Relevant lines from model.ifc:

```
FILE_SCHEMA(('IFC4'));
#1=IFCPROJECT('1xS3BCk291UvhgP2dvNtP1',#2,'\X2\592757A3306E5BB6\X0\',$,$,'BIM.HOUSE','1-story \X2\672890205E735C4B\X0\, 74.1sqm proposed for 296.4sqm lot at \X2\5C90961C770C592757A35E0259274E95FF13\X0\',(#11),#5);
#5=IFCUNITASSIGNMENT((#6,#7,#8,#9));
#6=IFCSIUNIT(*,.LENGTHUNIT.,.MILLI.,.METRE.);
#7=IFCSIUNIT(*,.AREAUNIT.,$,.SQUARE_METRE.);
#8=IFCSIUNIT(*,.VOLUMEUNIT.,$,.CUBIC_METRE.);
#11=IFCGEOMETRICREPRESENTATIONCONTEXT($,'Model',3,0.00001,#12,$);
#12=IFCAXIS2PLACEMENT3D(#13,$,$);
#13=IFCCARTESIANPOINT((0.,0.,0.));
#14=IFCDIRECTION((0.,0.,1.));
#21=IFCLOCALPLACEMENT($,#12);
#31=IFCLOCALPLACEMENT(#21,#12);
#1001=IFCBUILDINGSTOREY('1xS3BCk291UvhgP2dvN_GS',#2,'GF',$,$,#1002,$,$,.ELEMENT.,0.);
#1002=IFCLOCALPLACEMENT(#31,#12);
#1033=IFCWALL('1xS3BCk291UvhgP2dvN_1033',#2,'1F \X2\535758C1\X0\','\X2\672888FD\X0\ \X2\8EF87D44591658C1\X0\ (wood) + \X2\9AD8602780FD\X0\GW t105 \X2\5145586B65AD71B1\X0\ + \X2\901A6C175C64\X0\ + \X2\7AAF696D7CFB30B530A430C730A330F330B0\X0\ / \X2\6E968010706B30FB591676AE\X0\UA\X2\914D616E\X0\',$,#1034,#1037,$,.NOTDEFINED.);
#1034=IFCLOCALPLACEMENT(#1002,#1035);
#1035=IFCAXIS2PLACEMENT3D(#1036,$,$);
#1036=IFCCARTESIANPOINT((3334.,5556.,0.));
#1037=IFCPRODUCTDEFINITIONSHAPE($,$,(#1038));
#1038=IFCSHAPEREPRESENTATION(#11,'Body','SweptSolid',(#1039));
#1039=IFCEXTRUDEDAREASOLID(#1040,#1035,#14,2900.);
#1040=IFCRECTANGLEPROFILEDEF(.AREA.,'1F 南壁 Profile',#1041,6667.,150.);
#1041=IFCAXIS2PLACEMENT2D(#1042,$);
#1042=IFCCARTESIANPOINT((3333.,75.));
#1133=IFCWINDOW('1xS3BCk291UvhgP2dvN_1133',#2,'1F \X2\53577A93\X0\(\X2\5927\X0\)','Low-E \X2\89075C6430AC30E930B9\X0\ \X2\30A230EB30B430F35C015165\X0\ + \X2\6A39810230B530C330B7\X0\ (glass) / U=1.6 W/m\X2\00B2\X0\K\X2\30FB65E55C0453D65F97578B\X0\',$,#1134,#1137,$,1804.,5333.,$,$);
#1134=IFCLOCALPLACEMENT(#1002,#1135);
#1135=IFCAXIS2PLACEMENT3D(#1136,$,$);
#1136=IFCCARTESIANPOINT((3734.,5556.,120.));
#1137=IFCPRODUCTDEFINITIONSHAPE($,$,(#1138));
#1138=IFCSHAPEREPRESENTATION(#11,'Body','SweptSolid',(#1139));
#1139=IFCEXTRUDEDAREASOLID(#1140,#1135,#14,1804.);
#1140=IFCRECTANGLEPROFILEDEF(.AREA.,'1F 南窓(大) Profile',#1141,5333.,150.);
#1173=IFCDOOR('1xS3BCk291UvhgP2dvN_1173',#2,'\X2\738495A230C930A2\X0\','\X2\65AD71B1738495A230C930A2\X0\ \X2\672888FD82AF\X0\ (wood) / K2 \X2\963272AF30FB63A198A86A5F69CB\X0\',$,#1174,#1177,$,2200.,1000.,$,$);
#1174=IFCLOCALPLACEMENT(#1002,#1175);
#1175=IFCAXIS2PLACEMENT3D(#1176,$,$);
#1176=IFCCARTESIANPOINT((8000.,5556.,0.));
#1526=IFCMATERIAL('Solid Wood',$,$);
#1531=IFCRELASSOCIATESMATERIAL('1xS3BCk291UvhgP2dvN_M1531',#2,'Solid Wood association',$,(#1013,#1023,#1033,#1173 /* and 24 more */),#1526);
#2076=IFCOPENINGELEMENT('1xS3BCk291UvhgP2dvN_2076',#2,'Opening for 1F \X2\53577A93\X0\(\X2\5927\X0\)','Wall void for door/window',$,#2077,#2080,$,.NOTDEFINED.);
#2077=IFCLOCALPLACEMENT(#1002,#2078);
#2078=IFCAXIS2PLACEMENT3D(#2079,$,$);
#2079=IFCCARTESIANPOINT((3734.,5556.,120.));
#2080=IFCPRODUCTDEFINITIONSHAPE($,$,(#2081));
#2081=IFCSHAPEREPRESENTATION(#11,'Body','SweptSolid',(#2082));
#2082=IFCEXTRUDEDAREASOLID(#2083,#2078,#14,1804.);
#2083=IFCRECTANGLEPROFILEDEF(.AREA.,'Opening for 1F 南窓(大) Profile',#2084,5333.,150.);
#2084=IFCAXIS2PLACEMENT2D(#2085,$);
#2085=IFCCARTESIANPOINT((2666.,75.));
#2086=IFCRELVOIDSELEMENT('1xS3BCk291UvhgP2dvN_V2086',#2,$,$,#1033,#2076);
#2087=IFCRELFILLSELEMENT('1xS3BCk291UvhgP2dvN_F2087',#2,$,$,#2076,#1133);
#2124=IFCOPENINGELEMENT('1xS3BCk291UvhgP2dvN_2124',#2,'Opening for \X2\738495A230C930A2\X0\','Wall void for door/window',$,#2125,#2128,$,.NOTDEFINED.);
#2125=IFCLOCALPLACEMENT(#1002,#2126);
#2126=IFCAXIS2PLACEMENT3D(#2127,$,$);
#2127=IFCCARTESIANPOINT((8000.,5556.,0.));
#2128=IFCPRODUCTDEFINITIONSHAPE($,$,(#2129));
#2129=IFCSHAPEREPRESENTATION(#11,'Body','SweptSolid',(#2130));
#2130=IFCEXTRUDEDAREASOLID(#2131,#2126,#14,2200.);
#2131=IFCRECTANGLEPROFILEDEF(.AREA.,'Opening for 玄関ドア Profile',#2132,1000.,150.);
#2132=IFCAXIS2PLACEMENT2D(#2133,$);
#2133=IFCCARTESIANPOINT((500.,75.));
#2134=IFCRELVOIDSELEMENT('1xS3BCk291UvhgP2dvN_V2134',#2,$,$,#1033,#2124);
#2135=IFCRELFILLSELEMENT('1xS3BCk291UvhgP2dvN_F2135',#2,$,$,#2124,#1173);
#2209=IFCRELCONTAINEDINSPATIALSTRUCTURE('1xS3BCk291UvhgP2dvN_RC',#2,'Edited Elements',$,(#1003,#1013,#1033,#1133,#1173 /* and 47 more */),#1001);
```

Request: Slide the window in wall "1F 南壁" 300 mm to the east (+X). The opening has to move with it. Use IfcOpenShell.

```python
import ifcopenshell
import ifcopenshell.api.geometry
import ifcopenshell.util.placement
import ifcopenshell.util.unit

model = ifcopenshell.open("model.ifc")
unit_scale = ifcopenshell.util.unit.calculate_unit_scale(model)

window = model.by_guid("1xS3BCk291UvhgP2dvN_1133")
opening = window.FillsVoids[0].RelatingOpeningElement
wall = opening.VoidsElements[0].RelatingBuildingElement

wall_matrix = ifcopenshell.util.placement.get_local_placement(wall.ObjectPlacement)
shift = wall_matrix[:3, 0] * 0.3 / unit_scale
before = ifcopenshell.util.placement.get_local_placement(window.ObjectPlacement)[:3, 3].copy()

# The window is not placed relative to its opening, so move both.
for product in (opening, window):
    matrix = ifcopenshell.util.placement.get_local_placement(product.ObjectPlacement)
    matrix[:3, 3] += shift
    ifcopenshell.api.geometry.edit_object_placement(model, product=product, matrix=matrix, is_si=False)

after = ifcopenshell.util.placement.get_local_placement(window.ObjectPlacement)[:3, 3]
print("window moved by", (after - before).round(3) + 0.0)

model.write("model-out.ifc")
```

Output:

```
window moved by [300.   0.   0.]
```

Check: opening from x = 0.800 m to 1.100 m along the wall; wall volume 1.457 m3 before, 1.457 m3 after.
